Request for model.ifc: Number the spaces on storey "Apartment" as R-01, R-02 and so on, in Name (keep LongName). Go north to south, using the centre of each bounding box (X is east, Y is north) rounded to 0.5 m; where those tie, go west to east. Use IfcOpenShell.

First a look at what the model holds.

```python
import ifcopenshell
import ifcopenshell.util.element
import ifcopenshell.util.placement

model = ifcopenshell.open("model.ifc")
print(model.schema)
storey = next(s for s in model.by_type("IfcBuildingStorey") if s.Name == "Apartment")
spaces = [e for e in ifcopenshell.util.element.get_decomposition(storey) if e.is_a("IfcSpace")]
for e in sorted(spaces, key=lambda e: e.id()):
    origin = ifcopenshell.util.placement.get_local_placement(e.ObjectPlacement)[:3, 3]
    print(e.id(), e.Name, e.LongName, origin.round(2) + 0.0, sep=" | ")
```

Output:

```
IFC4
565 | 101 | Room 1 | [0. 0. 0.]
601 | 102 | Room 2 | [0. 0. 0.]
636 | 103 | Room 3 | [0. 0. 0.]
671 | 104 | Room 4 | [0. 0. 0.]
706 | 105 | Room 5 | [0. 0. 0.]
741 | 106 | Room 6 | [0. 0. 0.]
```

```python
import ifcopenshell
import ifcopenshell.geom
import ifcopenshell.util.element
import ifcopenshell.util.shape

model = ifcopenshell.open("model.ifc")
settings = ifcopenshell.geom.settings()
settings.set("use-world-coords", True)


def centre(element):
    shape = ifcopenshell.geom.create_shape(settings, element)
    return ifcopenshell.util.shape.get_bbox_centroid(shape.geometry)


storey = next(s for s in model.by_type("IfcBuildingStorey") if s.Name == "Apartment")
spaces = [e for e in ifcopenshell.util.element.get_decomposition(storey) if e.is_a("IfcSpace")]

# Insertion points can sit at a corner or the storey origin, so sort by the geometry (in metres).
centres = {e: centre(e) for e in spaces}
spaces.sort(key=lambda e: (-round(centres[e][1] / 0.5), centres[e][0]))

for i, e in enumerate(spaces, start=1):
    number = f"R-{i:02d}"
    e.Name = number
    print(e.id(), number)

model.write("model_v2.ifc")
```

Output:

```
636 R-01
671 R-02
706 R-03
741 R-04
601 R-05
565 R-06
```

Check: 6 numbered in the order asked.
